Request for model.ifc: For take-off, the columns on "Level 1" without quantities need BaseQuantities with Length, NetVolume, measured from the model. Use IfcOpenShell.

First a look at what the model holds.

```python
import ifcopenshell
import ifcopenshell.util.element
import ifcopenshell.util.unit

model = ifcopenshell.open("model.ifc")
print(model.schema)
for unit_type in ("LENGTHUNIT", "AREAUNIT", "VOLUMEUNIT"):
    print(unit_type, ifcopenshell.util.unit.calculate_unit_scale(model, unit_type))
storey = next(s for s in model.by_type("IfcBuildingStorey") if s.Name == "Level 1")
columns = [e for e in ifcopenshell.util.element.get_decomposition(storey) if e.is_a("IfcColumn")]
for e in sorted(columns, key=lambda e: e.id()):
    print(e.id(), e.is_a(), e.Name, list(ifcopenshell.util.element.get_psets(e, qtos_only=True)), sep=" | ")
```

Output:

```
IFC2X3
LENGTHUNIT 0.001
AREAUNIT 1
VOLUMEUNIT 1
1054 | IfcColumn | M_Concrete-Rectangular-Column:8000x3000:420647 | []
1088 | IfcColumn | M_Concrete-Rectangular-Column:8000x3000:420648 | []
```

```python
import ifcopenshell
import ifcopenshell.api.pset
import ifcopenshell.geom
import ifcopenshell.util.element
import ifcopenshell.util.shape
import ifcopenshell.util.unit

model = ifcopenshell.open("model.ifc")
unit_scale = ifcopenshell.util.unit.calculate_unit_scale(model)
volume_scale = ifcopenshell.util.unit.calculate_unit_scale(model, "VOLUMEUNIT")
settings = ifcopenshell.geom.settings()

storey = next(s for s in model.by_type("IfcBuildingStorey") if s.Name == "Level 1")
columns = [e for e in ifcopenshell.util.element.get_decomposition(storey) if e.is_a("IfcColumn")]

for e in sorted(columns, key=lambda e: e.id()):
    if ifcopenshell.util.element.get_psets(e, qtos_only=True, should_inherit=False):
        continue
    # Geometry comes back in metres, in the element's own axes.
    shape = ifcopenshell.geom.create_shape(settings, e)
    values = {
        "Length": ifcopenshell.util.shape.get_z(shape.geometry) / unit_scale,
        "NetVolume": ifcopenshell.util.shape.get_volume(shape.geometry) / volume_scale,
    }
    qto = ifcopenshell.api.pset.add_qto(model, product=e, name="BaseQuantities")
    ifcopenshell.api.pset.edit_qto(model, qto=qto, properties=values)
    print(e.id(), {k: round(v, 3) for k, v in values.items()})

model.write("model-out.ifc")
```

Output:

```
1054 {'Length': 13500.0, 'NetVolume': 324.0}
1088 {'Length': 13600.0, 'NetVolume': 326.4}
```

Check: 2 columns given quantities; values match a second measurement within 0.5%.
